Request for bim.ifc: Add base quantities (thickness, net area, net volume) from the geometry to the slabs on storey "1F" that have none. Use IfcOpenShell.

First a look at what the model holds.

```python
import ifcopenshell
import ifcopenshell.util.element
import ifcopenshell.util.unit

model = ifcopenshell.open("bim.ifc")
print(model.schema)
for unit_type in ("LENGTHUNIT", "AREAUNIT", "VOLUMEUNIT"):
    print(unit_type, ifcopenshell.util.unit.calculate_unit_scale(model, unit_type))
storey = next(s for s in model.by_type("IfcBuildingStorey") if s.Name == "1F")
slabs = [e for e in ifcopenshell.util.element.get_decomposition(storey) if e.is_a("IfcSlab")]
for e in sorted(slabs, key=lambda e: e.id()):
    print(e.id(), e.is_a(), e.Name, list(ifcopenshell.util.element.get_psets(e, qtos_only=True)), sep=" | ")
```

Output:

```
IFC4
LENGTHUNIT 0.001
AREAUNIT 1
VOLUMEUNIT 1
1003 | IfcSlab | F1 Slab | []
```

```python
import ifcopenshell
import ifcopenshell.api.pset
import ifcopenshell.geom
import ifcopenshell.util.element
import ifcopenshell.util.shape
import ifcopenshell.util.unit

model = ifcopenshell.open("bim.ifc")
unit_scale = ifcopenshell.util.unit.calculate_unit_scale(model)
area_scale = ifcopenshell.util.unit.calculate_unit_scale(model, "AREAUNIT")
volume_scale = ifcopenshell.util.unit.calculate_unit_scale(model, "VOLUMEUNIT")
settings = ifcopenshell.geom.settings()

storey = next(s for s in model.by_type("IfcBuildingStorey") if s.Name == "1F")
slabs = [e for e in ifcopenshell.util.element.get_decomposition(storey) if e.is_a("IfcSlab")]

for e in sorted(slabs, key=lambda e: e.id()):
    if ifcopenshell.util.element.get_psets(e, qtos_only=True, should_inherit=False):
        continue
    # Geometry comes back in metres, in the element's own axes.
    shape = ifcopenshell.geom.create_shape(settings, e)
    values = {
        "Width": ifcopenshell.util.shape.get_z(shape.geometry) / unit_scale,
        "NetArea": ifcopenshell.util.shape.get_footprint_area(shape.geometry) / area_scale,
        "NetVolume": ifcopenshell.util.shape.get_volume(shape.geometry) / volume_scale,
    }
    qto = ifcopenshell.api.pset.add_qto(model, product=e, name="Qto_SlabBaseQuantities")
    ifcopenshell.api.pset.edit_qto(model, qto=qto, properties=values)
    print(e.id(), {k: round(v, 3) for k, v in values.items()})

model.write("bim-out.ifc")
```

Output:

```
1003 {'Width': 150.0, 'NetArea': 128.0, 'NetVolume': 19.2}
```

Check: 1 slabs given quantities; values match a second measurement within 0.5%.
